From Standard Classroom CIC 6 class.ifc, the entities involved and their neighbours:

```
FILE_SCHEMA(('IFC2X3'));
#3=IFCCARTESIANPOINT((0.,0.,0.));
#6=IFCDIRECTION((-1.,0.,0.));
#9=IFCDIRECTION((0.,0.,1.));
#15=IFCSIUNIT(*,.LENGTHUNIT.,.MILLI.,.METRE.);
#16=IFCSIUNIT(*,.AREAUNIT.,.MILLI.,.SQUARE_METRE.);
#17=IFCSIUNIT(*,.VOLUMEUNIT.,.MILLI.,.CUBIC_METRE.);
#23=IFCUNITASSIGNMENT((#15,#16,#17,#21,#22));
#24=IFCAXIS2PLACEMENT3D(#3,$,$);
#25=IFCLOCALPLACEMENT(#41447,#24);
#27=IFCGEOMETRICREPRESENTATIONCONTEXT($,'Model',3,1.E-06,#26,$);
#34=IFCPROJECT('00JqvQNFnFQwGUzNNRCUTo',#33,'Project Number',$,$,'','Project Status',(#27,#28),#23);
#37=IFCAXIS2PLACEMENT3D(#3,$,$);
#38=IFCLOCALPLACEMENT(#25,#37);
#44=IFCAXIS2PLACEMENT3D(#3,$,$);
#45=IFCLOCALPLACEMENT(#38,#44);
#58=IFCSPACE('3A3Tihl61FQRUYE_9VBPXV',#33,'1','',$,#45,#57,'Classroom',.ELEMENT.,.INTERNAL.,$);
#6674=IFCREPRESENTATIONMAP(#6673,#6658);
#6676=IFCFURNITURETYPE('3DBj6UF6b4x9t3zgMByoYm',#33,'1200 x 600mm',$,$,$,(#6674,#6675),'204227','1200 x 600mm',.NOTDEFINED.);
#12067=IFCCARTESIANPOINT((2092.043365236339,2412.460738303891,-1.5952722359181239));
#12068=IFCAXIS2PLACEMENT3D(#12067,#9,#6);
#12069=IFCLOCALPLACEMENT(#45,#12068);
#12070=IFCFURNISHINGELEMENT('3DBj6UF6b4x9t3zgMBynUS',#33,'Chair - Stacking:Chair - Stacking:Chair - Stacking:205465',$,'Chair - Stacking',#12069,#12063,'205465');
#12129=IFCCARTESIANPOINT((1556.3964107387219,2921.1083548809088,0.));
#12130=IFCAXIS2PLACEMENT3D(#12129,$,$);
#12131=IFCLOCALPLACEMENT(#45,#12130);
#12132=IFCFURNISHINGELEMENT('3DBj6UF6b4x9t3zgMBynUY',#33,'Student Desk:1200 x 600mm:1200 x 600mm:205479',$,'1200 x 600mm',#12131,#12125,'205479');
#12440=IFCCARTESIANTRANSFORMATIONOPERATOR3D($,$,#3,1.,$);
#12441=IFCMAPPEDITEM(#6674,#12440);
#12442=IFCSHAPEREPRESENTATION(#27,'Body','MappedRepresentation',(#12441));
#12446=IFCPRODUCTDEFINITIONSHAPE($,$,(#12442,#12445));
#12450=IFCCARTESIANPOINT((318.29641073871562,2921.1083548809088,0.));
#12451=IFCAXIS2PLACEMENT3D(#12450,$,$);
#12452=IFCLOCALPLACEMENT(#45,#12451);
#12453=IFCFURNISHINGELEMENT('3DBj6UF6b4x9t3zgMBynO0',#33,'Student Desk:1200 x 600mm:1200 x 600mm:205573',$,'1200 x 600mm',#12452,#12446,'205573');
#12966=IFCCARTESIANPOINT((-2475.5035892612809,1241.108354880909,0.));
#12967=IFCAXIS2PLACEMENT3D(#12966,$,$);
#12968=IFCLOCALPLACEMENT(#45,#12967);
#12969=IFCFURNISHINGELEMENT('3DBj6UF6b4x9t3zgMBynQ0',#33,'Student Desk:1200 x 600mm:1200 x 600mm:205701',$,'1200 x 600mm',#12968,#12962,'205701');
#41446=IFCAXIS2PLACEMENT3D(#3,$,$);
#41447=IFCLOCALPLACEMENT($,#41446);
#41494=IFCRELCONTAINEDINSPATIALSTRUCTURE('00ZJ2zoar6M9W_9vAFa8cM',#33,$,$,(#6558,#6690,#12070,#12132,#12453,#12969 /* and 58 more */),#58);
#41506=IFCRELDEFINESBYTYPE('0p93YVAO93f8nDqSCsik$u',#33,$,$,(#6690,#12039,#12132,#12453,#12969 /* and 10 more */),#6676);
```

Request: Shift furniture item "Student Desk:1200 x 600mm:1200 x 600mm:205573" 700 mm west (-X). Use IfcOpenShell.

```python
import ifcopenshell
import ifcopenshell.api.geometry
import ifcopenshell.util.placement

model = ifcopenshell.open("Standard Classroom CIC 6 class.ifc")

item = model.by_guid("3DBj6UF6b4x9t3zgMBynO0")
matrix = ifcopenshell.util.placement.get_local_placement(item.ObjectPlacement)
matrix[0, 3] -= 700.0
ifcopenshell.api.geometry.edit_object_placement(model, product=item, matrix=matrix, is_si=False)

print(ifcopenshell.util.placement.get_local_placement(item.ObjectPlacement).round(3) + 0.0)

model.write("Standard Classroom CIC 6 class_v2.ifc")
```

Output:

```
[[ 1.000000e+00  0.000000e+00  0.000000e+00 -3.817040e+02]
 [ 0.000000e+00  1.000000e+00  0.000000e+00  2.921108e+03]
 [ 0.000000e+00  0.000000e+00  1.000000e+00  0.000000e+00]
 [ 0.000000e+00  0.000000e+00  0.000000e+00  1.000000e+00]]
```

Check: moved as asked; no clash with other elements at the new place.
